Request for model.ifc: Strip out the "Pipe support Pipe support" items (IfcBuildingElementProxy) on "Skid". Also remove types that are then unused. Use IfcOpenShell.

First a look at what the model holds.

```python
import ifcopenshell
import ifcopenshell.util.element

model = ifcopenshell.open("model.ifc")
print(model.schema)
storey = next(s for s in model.by_type("IfcBuildingStorey") if s.Name == "Skid")
proxies = [e for e in ifcopenshell.util.element.get_decomposition(storey) if e.is_a("IfcBuildingElementProxy")]
seen = {}
for e in proxies:
    element_type = ifcopenshell.util.element.get_type(e)
    name = element_type.Name if element_type not in (None, e) else None
    seen[name] = seen.get(name, 0) + 1
for name, count in sorted(seen.items(), key=str):
    print(count, "x", name)
```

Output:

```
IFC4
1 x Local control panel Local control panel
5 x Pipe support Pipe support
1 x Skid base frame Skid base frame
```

```python
import ifcopenshell
import ifcopenshell.api.root
import ifcopenshell.util.element

model = ifcopenshell.open("model.ifc")

storey = next(s for s in model.by_type("IfcBuildingStorey") if s.Name == "Skid")
proxies = [e for e in ifcopenshell.util.element.get_decomposition(storey) if e.is_a("IfcBuildingElementProxy")]
targets = [e for e in proxies if (t := ifcopenshell.util.element.get_type(e)) not in (None, e) and t.Name == "Pipe support Pipe support"]
types = {ifcopenshell.util.element.get_type(e) for e in targets} - {None, *targets}

for e in targets:
    ifcopenshell.api.root.remove_product(model, product=e)
print(len(targets), "removed")

unused = [t for t in types if not ifcopenshell.util.element.get_types(t)]
for t in unused:
    ifcopenshell.api.root.remove_product(model, product=t)
print(len(unused), "unused types removed")

model.write("model_v2.ifc")
```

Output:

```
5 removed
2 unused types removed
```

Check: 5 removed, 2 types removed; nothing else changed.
